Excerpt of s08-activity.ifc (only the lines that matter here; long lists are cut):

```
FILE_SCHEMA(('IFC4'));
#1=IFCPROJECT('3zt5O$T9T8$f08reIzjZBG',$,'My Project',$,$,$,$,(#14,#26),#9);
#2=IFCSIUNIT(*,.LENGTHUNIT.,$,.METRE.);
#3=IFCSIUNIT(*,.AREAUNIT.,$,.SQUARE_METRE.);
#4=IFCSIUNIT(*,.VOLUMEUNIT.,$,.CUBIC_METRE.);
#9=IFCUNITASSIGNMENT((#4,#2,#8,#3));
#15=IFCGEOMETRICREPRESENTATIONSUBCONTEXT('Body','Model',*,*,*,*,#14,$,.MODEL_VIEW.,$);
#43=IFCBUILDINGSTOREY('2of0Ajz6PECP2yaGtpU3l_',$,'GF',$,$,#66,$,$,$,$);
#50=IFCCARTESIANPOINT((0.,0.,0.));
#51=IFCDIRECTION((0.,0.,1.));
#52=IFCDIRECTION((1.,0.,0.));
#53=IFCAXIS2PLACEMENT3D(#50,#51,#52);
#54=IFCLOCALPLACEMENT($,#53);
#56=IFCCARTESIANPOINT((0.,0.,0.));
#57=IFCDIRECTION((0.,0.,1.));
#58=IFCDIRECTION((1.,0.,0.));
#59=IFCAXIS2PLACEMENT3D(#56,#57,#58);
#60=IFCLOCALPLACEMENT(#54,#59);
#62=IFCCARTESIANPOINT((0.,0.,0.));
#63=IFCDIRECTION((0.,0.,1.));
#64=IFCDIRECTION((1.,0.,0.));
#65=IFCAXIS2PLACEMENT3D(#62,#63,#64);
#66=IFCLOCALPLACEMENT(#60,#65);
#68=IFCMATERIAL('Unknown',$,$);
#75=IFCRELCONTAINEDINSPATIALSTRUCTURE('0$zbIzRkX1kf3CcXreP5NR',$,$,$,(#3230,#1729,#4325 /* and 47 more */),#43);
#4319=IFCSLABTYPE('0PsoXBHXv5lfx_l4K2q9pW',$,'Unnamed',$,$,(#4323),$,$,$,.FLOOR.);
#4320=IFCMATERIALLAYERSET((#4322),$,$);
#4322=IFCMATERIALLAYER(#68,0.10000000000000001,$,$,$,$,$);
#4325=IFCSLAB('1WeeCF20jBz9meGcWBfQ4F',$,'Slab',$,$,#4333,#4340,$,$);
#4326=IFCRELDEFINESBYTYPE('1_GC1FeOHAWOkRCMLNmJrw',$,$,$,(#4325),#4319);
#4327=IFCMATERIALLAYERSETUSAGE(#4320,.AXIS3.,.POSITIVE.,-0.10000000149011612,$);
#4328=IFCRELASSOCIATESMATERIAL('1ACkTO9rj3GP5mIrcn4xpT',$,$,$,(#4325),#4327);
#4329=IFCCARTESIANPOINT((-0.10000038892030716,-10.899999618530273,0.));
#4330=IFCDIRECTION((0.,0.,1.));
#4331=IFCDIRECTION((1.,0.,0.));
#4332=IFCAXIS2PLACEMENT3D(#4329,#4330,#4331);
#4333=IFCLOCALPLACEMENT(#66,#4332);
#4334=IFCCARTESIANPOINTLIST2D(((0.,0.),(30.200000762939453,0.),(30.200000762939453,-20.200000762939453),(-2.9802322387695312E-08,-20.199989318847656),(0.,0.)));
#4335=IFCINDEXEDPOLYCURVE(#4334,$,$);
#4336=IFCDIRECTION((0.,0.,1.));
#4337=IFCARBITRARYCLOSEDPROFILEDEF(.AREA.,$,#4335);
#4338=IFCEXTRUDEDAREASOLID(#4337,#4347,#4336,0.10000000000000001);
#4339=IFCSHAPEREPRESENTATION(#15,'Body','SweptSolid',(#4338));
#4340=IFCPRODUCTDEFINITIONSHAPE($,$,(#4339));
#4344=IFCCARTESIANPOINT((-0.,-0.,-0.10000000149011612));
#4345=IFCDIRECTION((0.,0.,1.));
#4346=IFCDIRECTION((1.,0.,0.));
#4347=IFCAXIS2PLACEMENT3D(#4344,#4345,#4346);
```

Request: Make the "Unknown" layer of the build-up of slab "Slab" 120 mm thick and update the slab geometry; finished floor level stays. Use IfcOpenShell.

```python
import ifcopenshell
import ifcopenshell.util.element
import ifcopenshell.util.representation
import ifcopenshell.util.unit

model = ifcopenshell.open("s08-activity.ifc")
unit_scale = ifcopenshell.util.unit.calculate_unit_scale(model)

layer_set = model.by_id(4320)
layer = next(l for l in layer_set.MaterialLayers if l.Material and l.Material.Name == "Unknown")
change = 0.12 / unit_scale - layer.LayerThickness
layer.LayerThickness += change

# Geometry does not follow the layer set by itself.
slabs = [e for e in ifcopenshell.util.element.get_elements_by_material(model, layer_set) if e.is_a("IfcSlab")]
for slab in sorted(slabs, key=lambda e: e.id()):
    body = ifcopenshell.util.representation.get_representation(slab, "Model", "Body")
    solid = body.Items[0]
    old_depth = solid.Depth
    solid.Depth += change
    # Extruded upwards: lower the start of the extrusion so the top stays.
    x, y, z = solid.Position.Location.Coordinates
    solid.Position.Location = model.createIfcCartesianPoint((x, y, z - change))
    print(slab.id(), f"{old_depth:g} -> {solid.Depth:g}")

# The layers are counted up from the underside, which has moved.
for usage in {ifcopenshell.util.element.get_material(slab) for slab in slabs}:
    usage.OffsetFromReferenceLine -= change

model.write("s08-activity_rev.ifc")
```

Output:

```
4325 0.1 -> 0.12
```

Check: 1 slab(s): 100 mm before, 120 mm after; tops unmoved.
